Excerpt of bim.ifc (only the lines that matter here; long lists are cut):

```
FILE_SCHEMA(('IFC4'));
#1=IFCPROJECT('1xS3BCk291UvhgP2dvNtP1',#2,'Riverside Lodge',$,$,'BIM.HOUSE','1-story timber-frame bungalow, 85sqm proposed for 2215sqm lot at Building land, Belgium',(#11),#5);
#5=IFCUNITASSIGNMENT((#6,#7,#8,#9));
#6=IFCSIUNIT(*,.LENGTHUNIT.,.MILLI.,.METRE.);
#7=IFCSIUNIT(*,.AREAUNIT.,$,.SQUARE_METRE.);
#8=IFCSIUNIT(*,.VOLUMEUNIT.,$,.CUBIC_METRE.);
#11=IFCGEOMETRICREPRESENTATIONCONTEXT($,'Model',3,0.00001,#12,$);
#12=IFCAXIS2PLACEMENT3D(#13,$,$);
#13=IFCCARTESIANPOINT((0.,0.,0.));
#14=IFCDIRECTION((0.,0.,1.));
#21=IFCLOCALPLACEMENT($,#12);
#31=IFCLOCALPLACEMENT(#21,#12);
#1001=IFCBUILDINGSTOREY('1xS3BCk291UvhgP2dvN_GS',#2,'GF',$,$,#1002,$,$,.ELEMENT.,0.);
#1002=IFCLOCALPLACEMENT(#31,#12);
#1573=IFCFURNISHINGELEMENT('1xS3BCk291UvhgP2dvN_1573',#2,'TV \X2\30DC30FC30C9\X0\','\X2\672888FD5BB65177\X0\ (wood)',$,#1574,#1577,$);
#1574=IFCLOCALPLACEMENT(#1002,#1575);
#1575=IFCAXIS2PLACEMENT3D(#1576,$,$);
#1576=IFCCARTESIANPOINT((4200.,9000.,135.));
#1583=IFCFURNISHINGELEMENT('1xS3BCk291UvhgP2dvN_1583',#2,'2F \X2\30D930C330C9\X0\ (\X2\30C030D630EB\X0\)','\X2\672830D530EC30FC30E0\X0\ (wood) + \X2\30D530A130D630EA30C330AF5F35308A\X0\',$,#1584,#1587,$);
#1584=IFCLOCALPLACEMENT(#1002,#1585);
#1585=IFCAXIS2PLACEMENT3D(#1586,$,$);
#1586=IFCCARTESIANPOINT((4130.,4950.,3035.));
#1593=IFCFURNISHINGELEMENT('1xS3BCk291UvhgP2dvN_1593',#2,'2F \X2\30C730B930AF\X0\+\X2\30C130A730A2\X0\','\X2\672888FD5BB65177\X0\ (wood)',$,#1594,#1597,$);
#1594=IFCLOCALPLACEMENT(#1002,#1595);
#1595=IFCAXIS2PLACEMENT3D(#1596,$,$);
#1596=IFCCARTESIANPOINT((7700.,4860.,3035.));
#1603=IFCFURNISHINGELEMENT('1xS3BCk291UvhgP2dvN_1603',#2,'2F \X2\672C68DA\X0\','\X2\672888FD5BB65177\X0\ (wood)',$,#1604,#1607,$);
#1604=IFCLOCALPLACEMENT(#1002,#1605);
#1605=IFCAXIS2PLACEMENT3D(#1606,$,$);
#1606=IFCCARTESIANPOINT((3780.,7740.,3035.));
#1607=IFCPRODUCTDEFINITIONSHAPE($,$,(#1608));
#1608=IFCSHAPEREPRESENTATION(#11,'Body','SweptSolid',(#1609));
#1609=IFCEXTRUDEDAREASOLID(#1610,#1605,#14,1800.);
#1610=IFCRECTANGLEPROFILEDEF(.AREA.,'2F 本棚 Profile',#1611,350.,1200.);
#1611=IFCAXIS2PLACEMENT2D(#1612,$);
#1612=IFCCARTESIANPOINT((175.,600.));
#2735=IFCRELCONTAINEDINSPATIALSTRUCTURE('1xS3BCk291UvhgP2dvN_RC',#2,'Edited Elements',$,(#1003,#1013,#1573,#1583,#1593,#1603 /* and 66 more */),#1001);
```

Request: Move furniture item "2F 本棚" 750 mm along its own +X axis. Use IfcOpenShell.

```python
import ifcopenshell
import ifcopenshell.api.geometry
import ifcopenshell.util.placement
import ifcopenshell.util.unit

model = ifcopenshell.open("bim.ifc")
unit_scale = ifcopenshell.util.unit.calculate_unit_scale(model)

item = model.by_guid("1xS3BCk291UvhgP2dvN_1603")
matrix = ifcopenshell.util.placement.get_local_placement(item.ObjectPlacement)
matrix[:3, 3] += matrix[:3, 0] * 0.75 / unit_scale
ifcopenshell.api.geometry.edit_object_placement(model, product=item, matrix=matrix, is_si=False)

print(ifcopenshell.util.placement.get_local_placement(item.ObjectPlacement).round(3) + 0.0)

model.write("bim-out.ifc")
```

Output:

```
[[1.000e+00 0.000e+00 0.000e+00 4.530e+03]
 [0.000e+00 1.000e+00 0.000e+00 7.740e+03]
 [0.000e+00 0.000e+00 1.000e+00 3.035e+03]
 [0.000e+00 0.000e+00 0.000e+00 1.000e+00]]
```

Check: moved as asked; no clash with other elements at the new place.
